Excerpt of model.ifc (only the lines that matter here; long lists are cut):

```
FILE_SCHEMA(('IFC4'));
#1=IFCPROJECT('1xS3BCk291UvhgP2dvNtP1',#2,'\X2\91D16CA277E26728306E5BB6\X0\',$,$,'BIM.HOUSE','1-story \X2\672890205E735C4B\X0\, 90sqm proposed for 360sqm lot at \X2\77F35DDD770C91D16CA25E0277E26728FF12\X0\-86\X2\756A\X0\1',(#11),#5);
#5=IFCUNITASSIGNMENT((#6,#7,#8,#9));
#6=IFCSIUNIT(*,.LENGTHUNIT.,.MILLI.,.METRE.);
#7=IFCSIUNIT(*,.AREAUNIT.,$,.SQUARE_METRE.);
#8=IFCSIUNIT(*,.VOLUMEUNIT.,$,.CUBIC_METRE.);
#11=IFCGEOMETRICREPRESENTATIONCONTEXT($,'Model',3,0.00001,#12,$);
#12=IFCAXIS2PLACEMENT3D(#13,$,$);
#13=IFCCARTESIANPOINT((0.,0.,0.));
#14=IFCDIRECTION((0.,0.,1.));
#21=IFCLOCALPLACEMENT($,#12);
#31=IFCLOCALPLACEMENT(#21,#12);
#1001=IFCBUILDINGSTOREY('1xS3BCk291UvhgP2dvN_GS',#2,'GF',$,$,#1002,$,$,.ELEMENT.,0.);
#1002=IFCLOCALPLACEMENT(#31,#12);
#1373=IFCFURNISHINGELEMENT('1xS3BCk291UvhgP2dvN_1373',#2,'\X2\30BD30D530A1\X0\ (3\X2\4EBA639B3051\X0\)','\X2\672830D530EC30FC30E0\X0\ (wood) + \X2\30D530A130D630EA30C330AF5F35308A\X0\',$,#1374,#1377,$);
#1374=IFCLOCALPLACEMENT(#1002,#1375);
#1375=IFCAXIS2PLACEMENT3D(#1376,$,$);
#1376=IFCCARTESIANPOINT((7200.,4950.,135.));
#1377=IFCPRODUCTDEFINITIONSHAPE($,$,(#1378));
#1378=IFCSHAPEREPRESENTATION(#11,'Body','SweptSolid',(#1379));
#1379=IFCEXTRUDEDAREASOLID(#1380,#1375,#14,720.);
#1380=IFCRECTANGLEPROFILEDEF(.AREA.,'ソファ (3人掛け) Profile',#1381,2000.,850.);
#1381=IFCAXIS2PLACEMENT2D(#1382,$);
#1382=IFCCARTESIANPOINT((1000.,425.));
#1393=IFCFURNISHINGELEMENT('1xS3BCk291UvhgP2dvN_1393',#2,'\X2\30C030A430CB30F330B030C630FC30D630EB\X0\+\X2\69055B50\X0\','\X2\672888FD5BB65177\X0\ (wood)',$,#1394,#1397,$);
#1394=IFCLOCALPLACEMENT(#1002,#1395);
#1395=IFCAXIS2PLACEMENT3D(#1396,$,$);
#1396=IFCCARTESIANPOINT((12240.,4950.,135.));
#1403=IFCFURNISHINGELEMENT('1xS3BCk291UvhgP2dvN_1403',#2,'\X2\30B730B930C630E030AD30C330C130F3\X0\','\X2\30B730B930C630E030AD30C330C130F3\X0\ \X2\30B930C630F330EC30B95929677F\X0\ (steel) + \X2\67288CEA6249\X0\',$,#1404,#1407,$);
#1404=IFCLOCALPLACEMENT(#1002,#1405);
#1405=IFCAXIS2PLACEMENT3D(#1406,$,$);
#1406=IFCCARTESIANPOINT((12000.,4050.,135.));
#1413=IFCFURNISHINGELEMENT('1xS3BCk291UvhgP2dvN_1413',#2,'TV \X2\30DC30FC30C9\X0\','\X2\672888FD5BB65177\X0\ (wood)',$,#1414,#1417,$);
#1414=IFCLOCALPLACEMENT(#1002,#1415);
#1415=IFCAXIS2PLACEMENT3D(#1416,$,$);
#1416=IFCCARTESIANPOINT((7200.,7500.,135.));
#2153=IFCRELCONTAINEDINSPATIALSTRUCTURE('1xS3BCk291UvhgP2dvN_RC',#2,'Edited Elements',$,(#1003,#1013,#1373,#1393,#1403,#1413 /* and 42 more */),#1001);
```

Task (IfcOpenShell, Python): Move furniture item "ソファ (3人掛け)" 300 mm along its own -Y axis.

```python
import ifcopenshell
import ifcopenshell.api.geometry
import ifcopenshell.util.placement
import ifcopenshell.util.unit

model = ifcopenshell.open("model.ifc")
unit_scale = ifcopenshell.util.unit.calculate_unit_scale(model)

item = model.by_guid("1xS3BCk291UvhgP2dvN_1373")
matrix = ifcopenshell.util.placement.get_local_placement(item.ObjectPlacement)
matrix[:3, 3] -= matrix[:3, 1] * 0.3 / unit_scale
ifcopenshell.api.geometry.edit_object_placement(model, product=item, matrix=matrix, is_si=False)

print(ifcopenshell.util.placement.get_local_placement(item.ObjectPlacement).round(3) + 0.0)

model.write("model_edited.ifc")
```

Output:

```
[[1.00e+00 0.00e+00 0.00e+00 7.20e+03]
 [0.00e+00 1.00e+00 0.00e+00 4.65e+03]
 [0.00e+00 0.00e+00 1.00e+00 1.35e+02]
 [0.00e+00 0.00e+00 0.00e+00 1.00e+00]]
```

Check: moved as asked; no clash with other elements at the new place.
